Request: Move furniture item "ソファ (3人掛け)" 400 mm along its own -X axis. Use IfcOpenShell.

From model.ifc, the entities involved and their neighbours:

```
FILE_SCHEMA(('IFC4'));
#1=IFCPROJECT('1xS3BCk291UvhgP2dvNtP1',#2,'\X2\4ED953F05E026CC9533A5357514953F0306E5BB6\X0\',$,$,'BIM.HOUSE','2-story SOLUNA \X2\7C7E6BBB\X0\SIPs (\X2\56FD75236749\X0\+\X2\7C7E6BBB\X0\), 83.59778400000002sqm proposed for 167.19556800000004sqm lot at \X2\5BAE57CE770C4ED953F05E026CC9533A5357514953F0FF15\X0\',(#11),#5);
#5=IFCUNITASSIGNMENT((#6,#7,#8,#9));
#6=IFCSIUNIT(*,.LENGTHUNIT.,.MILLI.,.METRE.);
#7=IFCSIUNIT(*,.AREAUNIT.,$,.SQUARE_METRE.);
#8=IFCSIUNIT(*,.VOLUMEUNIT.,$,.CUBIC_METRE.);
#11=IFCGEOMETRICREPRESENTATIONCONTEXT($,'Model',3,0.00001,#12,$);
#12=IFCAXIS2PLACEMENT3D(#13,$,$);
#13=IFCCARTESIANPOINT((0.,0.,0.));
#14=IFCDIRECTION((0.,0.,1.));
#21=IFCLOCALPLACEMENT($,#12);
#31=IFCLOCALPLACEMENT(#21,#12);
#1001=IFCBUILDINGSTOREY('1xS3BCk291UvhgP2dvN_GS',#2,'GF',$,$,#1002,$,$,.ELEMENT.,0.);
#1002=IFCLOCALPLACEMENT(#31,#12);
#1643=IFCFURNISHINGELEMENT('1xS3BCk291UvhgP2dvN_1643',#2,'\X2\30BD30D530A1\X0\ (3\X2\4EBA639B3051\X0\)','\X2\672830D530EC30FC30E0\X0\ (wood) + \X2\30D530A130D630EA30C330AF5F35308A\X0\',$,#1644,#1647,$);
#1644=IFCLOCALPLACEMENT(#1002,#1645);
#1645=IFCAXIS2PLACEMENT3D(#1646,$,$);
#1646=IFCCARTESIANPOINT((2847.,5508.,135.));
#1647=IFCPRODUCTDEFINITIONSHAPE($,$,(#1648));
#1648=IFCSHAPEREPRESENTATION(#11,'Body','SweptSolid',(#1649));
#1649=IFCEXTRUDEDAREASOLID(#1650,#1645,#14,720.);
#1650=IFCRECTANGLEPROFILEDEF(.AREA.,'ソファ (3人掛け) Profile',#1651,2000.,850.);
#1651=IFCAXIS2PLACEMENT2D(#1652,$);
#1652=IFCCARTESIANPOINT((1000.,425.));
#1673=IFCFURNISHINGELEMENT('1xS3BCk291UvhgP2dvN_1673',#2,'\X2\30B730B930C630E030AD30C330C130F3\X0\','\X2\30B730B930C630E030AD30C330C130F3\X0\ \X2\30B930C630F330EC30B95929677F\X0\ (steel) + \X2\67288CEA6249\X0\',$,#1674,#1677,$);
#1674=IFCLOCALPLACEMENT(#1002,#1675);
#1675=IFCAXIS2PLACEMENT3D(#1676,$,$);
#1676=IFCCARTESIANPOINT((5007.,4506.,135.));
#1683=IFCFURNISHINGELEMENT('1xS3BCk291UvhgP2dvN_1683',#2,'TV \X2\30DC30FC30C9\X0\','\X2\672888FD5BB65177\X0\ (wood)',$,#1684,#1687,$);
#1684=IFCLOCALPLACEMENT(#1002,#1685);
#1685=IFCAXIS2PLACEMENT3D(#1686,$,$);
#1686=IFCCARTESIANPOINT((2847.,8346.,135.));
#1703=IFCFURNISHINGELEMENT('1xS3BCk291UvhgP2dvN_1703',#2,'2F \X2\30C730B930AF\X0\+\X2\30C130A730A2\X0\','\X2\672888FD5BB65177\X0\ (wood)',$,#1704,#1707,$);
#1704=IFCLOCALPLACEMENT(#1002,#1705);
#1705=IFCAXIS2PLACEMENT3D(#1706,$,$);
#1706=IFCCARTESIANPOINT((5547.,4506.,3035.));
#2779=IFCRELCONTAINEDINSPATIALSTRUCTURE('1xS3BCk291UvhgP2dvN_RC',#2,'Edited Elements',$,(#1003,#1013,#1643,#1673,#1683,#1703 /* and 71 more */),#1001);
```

```python
import ifcopenshell
import ifcopenshell.api.geometry
import ifcopenshell.util.placement
import ifcopenshell.util.unit

model = ifcopenshell.open("model.ifc")
unit_scale = ifcopenshell.util.unit.calculate_unit_scale(model)

item = model.by_id(1643)
matrix = ifcopenshell.util.placement.get_local_placement(item.ObjectPlacement)
matrix[:3, 3] -= matrix[:3, 0] * 0.4 / unit_scale
ifcopenshell.api.geometry.edit_object_placement(model, product=item, matrix=matrix, is_si=False)

print(ifcopenshell.util.placement.get_local_placement(item.ObjectPlacement).round(3) + 0.0)

model.write("model_edited.ifc")
```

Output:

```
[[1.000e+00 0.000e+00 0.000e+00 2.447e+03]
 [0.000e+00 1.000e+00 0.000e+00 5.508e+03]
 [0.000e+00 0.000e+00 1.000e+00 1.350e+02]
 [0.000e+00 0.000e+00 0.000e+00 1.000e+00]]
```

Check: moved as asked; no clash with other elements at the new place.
